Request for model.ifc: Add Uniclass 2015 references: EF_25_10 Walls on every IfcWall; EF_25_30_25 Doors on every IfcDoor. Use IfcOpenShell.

First a look at what the model holds.

```python
import ifcopenshell

model = ifcopenshell.open("model.ifc")
print(model.schema)
print("classifications:", [c.Name for c in model.by_type("IfcClassification")])
for ifc_class in ("IfcDoor", "IfcRoof", "IfcStair", "IfcWall", "IfcWindow"):
    print(ifc_class, len(model.by_type(ifc_class)))
```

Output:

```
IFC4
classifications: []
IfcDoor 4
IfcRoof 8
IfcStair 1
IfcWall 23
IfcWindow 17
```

```python
import ifcopenshell
import ifcopenshell.api.classification

model = ifcopenshell.open("model.ifc")

system = ifcopenshell.api.classification.add_classification(model, classification="Uniclass 2015")

codes = {
    "IfcWall": ("EF_25_10", "Walls"),
    "IfcDoor": ("EF_25_30_25", "Doors"),
}
for ifc_class, (code, name) in codes.items():
    products = model.by_type(ifc_class)
    ifcopenshell.api.classification.add_reference(
        model, products=products, classification=system, identification=code, name=name
    )
    print(code, len(products))

model.write("model_v2.ifc")
```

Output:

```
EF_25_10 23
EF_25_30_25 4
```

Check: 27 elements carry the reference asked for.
